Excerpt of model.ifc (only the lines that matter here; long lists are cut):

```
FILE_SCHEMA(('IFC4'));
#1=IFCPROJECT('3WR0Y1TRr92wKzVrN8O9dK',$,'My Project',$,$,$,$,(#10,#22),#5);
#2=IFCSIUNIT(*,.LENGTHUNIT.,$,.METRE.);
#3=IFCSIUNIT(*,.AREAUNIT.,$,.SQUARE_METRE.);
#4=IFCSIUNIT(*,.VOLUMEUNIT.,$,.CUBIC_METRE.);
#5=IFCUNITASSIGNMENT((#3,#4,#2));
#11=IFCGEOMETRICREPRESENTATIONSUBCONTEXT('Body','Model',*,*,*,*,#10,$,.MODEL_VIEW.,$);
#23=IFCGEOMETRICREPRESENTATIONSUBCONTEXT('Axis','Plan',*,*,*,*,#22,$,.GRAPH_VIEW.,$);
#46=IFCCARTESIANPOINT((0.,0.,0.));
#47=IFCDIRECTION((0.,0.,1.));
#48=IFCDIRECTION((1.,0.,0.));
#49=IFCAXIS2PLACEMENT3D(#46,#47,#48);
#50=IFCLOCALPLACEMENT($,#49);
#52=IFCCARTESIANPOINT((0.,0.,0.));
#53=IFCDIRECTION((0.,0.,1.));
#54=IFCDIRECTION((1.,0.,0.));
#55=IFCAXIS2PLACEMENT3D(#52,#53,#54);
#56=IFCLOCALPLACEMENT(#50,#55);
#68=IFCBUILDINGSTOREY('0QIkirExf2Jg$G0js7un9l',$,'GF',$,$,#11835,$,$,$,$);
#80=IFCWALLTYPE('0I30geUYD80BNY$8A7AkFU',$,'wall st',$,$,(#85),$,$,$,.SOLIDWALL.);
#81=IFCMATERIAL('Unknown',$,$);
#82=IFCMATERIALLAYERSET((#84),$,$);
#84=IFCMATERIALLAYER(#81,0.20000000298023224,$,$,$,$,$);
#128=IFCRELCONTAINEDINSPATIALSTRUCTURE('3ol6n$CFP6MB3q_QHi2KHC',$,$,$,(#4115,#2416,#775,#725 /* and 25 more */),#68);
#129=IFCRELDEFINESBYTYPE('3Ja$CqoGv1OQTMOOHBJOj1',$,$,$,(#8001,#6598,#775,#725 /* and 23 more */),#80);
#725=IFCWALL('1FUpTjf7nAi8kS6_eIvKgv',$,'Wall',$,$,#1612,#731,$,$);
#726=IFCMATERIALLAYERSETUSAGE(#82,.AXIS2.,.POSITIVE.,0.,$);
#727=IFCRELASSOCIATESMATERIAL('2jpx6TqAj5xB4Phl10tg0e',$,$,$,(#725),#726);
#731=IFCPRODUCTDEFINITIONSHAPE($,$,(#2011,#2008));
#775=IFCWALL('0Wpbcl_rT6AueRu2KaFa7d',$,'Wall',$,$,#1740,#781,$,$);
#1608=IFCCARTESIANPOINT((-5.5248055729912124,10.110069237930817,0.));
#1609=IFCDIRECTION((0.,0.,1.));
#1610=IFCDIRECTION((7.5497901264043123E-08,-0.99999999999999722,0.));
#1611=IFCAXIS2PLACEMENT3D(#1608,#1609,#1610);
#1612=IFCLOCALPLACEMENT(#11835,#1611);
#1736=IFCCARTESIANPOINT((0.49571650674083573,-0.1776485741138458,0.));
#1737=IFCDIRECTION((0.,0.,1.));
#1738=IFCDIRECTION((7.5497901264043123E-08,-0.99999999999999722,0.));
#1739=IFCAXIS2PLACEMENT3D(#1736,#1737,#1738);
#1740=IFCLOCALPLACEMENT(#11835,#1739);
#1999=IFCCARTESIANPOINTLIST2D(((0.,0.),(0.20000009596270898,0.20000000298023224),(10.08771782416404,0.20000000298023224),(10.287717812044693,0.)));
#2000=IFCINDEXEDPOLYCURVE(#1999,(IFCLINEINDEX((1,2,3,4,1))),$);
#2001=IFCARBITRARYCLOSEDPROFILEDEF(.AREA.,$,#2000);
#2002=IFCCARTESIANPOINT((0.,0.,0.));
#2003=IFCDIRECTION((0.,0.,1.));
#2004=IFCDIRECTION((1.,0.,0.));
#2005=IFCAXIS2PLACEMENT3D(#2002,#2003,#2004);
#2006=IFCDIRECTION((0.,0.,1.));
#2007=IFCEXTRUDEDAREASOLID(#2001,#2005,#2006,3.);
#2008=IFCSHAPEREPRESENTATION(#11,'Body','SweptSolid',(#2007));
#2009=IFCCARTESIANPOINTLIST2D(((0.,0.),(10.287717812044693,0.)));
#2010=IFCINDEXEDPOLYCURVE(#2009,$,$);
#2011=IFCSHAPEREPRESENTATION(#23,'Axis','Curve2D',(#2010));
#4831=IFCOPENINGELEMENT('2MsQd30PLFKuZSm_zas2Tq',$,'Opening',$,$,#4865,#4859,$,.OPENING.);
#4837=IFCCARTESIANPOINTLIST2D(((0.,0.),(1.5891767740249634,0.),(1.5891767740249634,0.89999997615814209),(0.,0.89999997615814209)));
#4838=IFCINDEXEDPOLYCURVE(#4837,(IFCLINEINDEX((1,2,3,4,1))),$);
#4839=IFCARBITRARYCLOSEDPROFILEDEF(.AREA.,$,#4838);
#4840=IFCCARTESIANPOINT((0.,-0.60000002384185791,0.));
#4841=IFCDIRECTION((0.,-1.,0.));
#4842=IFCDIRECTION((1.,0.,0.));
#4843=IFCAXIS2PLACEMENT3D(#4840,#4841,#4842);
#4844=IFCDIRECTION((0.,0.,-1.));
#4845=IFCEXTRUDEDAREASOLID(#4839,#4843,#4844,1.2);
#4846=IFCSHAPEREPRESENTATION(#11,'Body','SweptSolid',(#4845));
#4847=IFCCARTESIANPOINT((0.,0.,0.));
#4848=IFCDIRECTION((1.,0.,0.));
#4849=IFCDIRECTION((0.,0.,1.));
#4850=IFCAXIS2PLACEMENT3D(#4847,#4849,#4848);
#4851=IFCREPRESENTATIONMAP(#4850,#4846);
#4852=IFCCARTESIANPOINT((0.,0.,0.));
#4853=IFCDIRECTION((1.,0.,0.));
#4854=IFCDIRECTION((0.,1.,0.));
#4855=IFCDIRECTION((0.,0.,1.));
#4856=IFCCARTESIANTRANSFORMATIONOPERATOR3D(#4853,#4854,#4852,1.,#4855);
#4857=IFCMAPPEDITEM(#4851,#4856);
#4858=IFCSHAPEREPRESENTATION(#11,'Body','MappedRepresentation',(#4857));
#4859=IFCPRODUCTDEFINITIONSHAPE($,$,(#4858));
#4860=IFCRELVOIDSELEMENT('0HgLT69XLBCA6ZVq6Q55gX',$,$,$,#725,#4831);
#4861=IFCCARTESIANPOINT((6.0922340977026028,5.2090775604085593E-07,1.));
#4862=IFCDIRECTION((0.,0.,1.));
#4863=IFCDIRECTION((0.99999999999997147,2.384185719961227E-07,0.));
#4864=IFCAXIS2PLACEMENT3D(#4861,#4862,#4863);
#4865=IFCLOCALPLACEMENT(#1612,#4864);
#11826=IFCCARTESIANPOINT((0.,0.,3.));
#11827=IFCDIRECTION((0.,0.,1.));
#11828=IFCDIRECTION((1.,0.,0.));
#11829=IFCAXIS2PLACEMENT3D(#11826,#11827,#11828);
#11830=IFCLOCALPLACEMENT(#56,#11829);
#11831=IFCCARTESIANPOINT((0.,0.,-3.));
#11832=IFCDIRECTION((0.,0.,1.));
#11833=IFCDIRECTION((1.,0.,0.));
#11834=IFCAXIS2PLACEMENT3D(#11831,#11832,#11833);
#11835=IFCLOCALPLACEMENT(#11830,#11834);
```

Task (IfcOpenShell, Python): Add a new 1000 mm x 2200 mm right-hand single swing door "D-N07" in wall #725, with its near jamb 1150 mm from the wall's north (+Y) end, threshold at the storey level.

```python
import numpy as np
import ifcopenshell
import ifcopenshell.api.feature
import ifcopenshell.api.geometry
import ifcopenshell.api.root
import ifcopenshell.api.spatial
import ifcopenshell.geom
import ifcopenshell.util.element
import ifcopenshell.util.placement
import ifcopenshell.util.representation
import ifcopenshell.util.shape
import ifcopenshell.util.unit

model = ifcopenshell.open("model.ifc")
unit_scale = ifcopenshell.util.unit.calculate_unit_scale(model)
settings = ifcopenshell.geom.settings()


def volume(element):
    """Net volume in cubic metres, openings subtracted."""
    shape = ifcopenshell.geom.create_shape(settings, element)
    return ifcopenshell.util.shape.get_volume(shape.geometry)


wall = model.by_guid("1FUpTjf7nAi8kS6_eIvKgv")
storey = ifcopenshell.util.element.get_container(wall, ifc_class="IfcBuildingStorey")
context = ifcopenshell.util.representation.get_context(model, "Model", "Body", "MODEL_VIEW")
before = volume(wall)

width, height, from_end, sill = 1, 2.2, 1.15, 0.0  # metres

# The wall runs along its own X axis, and the end named is its -X end.
wall_shape = ifcopenshell.geom.create_shape(settings, wall)
x, y, z = ifcopenshell.util.shape.get_vertices(wall_shape.geometry).T
start = x.min() + from_end
face, thickness = float(y.min()), float(y.max() - y.min())
wall_matrix = ifcopenshell.util.placement.get_local_placement(wall.ObjectPlacement)
level = ifcopenshell.util.placement.get_local_placement(storey.ObjectPlacement)[2, 3]


def in_wall(x, y):
    """Placement at x, y metres in the wall's axes, at sill height."""
    matrix = wall_matrix.copy()
    matrix[:, 3] = wall_matrix @ np.array([x / unit_scale, y / unit_scale, 0.0, 1.0])
    matrix[2, 3] = level + sill / unit_scale
    return matrix


# Opening: a box that overshoots both wall faces by 50 mm.
opening = ifcopenshell.api.root.create_entity(model, ifc_class="IfcOpeningElement", predefined_type="OPENING")
box = ifcopenshell.api.geometry.add_wall_representation(
    model, context=context, length=width, height=height, thickness=thickness + 0.1
)
ifcopenshell.api.geometry.assign_representation(model, product=opening, representation=box)
ifcopenshell.api.geometry.edit_object_placement(model, product=opening, matrix=in_wall(start, face - 0.05), is_si=False)
ifcopenshell.api.feature.add_feature(model, feature=opening, element=wall)

door = ifcopenshell.api.root.create_entity(model, ifc_class="IfcDoor", name="D-N07", predefined_type="DOOR")
door.OverallWidth, door.OverallHeight = width / unit_scale, height / unit_scale
door.OperationType = "SINGLE_SWING_RIGHT"
body = ifcopenshell.api.geometry.add_door_representation(
    model,
    context=context,
    overall_width=door.OverallWidth,
    overall_height=door.OverallHeight,
    operation_type="SINGLE_SWING_RIGHT",
    lining_properties={"LiningDepth": thickness / unit_scale, "ThresholdDepth": thickness / unit_scale},
)
ifcopenshell.api.geometry.assign_representation(model, product=door, representation=body)
ifcopenshell.api.spatial.assign_container(model, products=[door], relating_structure=storey)
ifcopenshell.api.feature.add_filling(model, opening=opening, element=door)

# The lining spans the wall, so the door starts at the wall face.
ifcopenshell.api.geometry.edit_object_placement(model, product=door, matrix=in_wall(start, face), is_si=False)

after = volume(wall)

print(f"wall volume {before:.3f} -> {after:.3f} m3")

model.write("model_v2.ifc")
```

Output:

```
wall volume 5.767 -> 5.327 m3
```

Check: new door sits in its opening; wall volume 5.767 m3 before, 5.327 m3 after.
